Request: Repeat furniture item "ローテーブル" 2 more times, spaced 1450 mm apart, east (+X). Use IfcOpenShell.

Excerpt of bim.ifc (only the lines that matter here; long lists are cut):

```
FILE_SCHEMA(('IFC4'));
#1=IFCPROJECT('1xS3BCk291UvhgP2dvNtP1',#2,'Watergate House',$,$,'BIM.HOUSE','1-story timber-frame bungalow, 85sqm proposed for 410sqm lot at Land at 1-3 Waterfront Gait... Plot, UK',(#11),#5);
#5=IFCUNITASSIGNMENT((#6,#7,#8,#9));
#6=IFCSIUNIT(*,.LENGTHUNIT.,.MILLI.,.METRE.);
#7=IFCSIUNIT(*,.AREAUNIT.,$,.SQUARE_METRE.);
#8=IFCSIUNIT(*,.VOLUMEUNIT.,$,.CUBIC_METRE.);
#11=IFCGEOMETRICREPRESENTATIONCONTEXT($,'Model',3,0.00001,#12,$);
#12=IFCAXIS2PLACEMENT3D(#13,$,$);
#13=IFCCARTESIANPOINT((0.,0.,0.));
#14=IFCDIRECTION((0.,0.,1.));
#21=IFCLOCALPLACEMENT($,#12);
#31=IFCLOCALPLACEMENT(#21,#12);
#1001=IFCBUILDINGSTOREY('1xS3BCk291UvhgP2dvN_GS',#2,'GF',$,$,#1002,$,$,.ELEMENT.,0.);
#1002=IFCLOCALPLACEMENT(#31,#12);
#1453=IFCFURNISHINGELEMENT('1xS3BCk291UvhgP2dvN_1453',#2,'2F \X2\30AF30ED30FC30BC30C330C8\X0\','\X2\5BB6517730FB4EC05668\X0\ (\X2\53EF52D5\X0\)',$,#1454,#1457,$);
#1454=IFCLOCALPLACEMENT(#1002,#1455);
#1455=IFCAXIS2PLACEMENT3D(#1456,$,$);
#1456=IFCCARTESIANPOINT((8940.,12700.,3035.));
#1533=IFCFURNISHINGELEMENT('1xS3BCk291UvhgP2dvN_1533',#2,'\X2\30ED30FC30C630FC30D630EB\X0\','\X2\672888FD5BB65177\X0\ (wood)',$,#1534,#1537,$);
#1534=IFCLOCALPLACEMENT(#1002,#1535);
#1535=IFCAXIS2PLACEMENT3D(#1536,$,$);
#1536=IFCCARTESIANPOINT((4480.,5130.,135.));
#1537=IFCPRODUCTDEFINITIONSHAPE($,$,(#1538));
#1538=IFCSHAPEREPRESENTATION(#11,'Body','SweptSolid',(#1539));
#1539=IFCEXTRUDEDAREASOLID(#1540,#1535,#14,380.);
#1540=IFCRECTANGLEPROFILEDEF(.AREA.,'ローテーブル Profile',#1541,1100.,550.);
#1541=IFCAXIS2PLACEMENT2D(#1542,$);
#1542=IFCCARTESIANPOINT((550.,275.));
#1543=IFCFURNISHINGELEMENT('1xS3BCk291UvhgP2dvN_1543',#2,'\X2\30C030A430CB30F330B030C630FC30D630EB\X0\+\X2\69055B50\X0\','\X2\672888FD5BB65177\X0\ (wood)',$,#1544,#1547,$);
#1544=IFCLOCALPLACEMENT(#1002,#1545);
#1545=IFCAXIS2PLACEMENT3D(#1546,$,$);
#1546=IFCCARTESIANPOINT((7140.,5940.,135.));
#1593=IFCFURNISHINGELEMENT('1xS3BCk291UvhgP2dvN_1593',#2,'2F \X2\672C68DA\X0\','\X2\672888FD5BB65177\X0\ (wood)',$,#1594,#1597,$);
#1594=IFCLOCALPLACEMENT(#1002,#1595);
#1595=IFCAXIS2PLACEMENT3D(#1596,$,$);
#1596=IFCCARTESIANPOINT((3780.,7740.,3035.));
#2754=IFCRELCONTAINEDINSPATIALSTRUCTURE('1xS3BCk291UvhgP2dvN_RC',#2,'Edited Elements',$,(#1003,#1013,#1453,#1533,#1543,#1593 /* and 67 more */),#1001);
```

```python
import numpy as np
import ifcopenshell
import ifcopenshell.api.geometry
import ifcopenshell.api.root
import ifcopenshell.util.element
import ifcopenshell.util.placement

model = ifcopenshell.open("bim.ifc")


def reuse_history(source, copy):
    """copy_class also copies each property set's owner history, people and application; keep the originals."""
    for rel in copy.IsDefinedBy:
        if rel.is_a("IfcRelDefinesByProperties") and (history := rel.RelatingPropertyDefinition.OwnerHistory):
            rel.RelatingPropertyDefinition.OwnerHistory = source.OwnerHistory
            ifcopenshell.util.element.remove_deep2(model, history)


source = model.by_guid("1xS3BCk291UvhgP2dvN_1533")
base = ifcopenshell.util.placement.get_local_placement(source.ObjectPlacement)
step = np.array([1.0, 0.0, 0.0]) * 1450.0

for i in range(1, 3):
    copy = ifcopenshell.api.root.copy_class(model, product=source)
    copy.Representation = ifcopenshell.util.element.copy_deep(
        model, source.Representation, exclude=["IfcGeometricRepresentationContext", "IfcRepresentationMap"]
    )
    reuse_history(source, copy)
    matrix = base.copy()
    matrix[:3, 3] += i * step
    print("added at", matrix[:3, 3].round(3) + 0.0)
    ifcopenshell.api.geometry.edit_object_placement(model, product=copy, matrix=matrix, is_si=False)

model.write("bim_updated.ifc")
```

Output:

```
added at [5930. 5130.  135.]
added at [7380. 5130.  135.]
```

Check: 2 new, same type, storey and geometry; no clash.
